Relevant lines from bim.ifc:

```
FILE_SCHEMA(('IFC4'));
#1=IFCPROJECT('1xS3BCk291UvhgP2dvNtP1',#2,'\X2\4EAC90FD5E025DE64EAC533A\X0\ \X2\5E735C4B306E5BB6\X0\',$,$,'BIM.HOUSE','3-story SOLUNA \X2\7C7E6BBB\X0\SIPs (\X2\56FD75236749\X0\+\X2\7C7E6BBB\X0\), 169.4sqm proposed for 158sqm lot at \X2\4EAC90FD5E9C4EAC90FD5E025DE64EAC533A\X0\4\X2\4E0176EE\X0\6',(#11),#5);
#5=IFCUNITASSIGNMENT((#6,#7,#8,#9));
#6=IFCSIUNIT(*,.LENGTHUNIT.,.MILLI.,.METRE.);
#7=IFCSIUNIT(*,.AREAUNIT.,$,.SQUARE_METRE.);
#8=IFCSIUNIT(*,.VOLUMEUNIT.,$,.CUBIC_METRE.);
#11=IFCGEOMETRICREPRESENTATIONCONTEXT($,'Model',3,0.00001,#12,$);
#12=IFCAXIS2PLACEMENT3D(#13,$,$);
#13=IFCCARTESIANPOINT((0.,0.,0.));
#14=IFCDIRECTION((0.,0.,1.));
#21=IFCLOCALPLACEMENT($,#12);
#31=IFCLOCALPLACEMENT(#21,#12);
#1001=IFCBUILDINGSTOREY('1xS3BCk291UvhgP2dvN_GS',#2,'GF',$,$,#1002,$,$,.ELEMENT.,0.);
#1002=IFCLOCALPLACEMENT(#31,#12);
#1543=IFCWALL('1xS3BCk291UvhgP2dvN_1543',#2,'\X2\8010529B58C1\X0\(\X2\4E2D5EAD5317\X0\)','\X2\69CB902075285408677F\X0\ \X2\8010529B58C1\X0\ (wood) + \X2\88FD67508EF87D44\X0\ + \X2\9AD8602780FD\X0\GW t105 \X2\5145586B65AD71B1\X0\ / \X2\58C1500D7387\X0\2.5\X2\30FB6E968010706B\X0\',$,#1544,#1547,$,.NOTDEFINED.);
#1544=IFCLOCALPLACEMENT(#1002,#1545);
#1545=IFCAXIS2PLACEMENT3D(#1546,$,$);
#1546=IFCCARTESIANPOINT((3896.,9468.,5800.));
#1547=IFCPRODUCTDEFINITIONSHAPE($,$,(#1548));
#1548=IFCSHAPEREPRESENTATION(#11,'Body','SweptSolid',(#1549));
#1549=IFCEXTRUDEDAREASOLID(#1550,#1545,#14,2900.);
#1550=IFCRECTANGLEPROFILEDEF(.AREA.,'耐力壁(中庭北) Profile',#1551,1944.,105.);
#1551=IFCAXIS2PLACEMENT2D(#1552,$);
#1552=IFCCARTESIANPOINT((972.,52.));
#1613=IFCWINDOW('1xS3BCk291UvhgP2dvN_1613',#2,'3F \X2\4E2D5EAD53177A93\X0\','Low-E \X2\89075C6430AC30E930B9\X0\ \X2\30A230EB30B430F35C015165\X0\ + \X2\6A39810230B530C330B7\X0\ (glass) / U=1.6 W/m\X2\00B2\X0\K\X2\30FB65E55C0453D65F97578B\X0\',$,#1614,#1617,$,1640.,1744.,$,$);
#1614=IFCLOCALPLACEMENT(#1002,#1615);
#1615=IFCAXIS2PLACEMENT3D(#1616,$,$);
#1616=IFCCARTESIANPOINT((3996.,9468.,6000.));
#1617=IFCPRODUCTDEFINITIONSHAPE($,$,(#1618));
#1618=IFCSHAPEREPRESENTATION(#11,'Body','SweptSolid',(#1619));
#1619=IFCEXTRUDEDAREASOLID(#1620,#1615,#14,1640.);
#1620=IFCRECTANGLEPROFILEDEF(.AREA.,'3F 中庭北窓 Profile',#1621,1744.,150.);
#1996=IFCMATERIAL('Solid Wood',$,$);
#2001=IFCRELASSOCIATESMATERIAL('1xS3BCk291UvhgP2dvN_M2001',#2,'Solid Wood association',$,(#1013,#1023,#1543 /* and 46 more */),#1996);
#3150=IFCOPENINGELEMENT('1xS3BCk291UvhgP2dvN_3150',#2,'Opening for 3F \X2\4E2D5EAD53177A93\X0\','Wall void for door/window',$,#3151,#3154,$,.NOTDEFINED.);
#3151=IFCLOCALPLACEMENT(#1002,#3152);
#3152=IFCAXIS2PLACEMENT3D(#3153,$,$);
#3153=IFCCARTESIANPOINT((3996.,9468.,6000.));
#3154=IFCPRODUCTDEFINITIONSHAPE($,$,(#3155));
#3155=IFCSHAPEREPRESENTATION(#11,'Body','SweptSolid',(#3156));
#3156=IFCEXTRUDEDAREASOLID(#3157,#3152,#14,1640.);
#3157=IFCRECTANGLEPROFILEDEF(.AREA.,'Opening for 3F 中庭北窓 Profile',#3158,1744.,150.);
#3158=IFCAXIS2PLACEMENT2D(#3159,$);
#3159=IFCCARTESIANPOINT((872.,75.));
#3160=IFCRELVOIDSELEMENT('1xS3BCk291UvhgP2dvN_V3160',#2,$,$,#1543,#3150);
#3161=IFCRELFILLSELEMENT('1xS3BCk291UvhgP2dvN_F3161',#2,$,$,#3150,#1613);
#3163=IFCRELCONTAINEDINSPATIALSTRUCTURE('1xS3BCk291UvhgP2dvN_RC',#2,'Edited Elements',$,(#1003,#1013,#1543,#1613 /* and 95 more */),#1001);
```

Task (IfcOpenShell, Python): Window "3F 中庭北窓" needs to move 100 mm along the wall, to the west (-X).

```python
import ifcopenshell
import ifcopenshell.api.geometry
import ifcopenshell.util.placement

model = ifcopenshell.open("bim.ifc")

window = model.by_id(1613)
opening = window.FillsVoids[0].RelatingOpeningElement
wall = opening.VoidsElements[0].RelatingBuildingElement

wall_matrix = ifcopenshell.util.placement.get_local_placement(wall.ObjectPlacement)
shift = wall_matrix[:3, 0] * -100.0
before = ifcopenshell.util.placement.get_local_placement(window.ObjectPlacement)[:3, 3].copy()

# The window is not placed relative to its opening, so move both.
for product in (opening, window):
    matrix = ifcopenshell.util.placement.get_local_placement(product.ObjectPlacement)
    matrix[:3, 3] += shift
    ifcopenshell.api.geometry.edit_object_placement(model, product=product, matrix=matrix, is_si=False)

after = ifcopenshell.util.placement.get_local_placement(window.ObjectPlacement)[:3, 3]
print("window moved by", (after - before).round(3) + 0.0)

model.write("bim_updated.ifc")
```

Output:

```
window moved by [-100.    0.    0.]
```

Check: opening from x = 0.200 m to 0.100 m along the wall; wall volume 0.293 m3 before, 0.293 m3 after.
